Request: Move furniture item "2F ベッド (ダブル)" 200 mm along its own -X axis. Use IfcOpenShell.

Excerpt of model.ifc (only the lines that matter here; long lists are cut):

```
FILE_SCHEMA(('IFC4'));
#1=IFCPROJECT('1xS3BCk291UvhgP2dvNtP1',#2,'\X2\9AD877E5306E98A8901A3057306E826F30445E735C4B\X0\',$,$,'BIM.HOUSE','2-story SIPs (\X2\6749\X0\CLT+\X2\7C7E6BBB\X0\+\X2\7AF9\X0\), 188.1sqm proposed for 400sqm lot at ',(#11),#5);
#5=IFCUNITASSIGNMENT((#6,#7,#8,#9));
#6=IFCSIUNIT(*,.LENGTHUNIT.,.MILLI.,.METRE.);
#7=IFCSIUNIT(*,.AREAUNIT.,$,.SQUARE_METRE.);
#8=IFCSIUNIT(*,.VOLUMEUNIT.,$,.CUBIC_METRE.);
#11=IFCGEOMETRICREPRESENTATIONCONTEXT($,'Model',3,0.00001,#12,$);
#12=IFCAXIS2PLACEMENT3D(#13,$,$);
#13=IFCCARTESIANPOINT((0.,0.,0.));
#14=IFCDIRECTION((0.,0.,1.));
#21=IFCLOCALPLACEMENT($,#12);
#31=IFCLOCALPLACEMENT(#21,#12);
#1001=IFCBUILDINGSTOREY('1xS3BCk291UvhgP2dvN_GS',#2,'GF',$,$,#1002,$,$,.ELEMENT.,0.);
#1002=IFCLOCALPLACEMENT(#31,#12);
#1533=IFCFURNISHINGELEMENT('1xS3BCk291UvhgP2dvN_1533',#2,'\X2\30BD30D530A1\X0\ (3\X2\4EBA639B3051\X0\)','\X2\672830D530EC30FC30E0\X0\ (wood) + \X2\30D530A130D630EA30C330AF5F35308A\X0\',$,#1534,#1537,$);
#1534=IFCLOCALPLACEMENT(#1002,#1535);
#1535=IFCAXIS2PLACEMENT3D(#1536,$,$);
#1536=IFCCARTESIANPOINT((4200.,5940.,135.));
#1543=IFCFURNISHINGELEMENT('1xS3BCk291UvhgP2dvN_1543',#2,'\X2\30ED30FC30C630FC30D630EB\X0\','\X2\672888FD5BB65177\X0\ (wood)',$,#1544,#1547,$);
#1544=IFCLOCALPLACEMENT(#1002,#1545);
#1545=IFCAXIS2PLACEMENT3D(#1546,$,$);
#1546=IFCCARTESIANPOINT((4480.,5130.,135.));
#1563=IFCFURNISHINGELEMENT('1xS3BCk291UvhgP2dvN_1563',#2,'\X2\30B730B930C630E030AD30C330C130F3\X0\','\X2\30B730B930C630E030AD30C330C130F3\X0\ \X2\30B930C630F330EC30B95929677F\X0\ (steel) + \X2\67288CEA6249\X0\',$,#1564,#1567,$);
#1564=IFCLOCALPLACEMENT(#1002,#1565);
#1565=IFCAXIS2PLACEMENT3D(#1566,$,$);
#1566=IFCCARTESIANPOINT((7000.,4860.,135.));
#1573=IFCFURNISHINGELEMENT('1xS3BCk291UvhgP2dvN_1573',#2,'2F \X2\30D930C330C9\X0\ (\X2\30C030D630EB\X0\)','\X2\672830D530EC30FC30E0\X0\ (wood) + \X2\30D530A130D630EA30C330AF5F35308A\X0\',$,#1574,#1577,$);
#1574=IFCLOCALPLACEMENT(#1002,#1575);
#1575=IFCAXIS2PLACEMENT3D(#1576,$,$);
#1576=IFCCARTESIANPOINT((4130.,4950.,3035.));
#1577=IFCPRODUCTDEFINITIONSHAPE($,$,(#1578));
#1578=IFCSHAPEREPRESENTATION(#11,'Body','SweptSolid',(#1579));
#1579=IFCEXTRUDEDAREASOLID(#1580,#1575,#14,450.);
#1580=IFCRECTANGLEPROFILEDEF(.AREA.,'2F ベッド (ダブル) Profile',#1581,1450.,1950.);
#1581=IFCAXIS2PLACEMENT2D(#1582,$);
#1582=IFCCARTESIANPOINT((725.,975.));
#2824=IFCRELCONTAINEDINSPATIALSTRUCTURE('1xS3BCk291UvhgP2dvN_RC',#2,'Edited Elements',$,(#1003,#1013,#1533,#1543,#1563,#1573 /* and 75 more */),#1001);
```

```python
import ifcopenshell
import ifcopenshell.api.geometry
import ifcopenshell.util.placement

model = ifcopenshell.open("model.ifc")

item = model.by_guid("1xS3BCk291UvhgP2dvN_1573")
matrix = ifcopenshell.util.placement.get_local_placement(item.ObjectPlacement)
matrix[:3, 3] -= matrix[:3, 0] * 200.0
ifcopenshell.api.geometry.edit_object_placement(model, product=item, matrix=matrix, is_si=False)

print(ifcopenshell.util.placement.get_local_placement(item.ObjectPlacement).round(3) + 0.0)

model.write("model_v2.ifc")
```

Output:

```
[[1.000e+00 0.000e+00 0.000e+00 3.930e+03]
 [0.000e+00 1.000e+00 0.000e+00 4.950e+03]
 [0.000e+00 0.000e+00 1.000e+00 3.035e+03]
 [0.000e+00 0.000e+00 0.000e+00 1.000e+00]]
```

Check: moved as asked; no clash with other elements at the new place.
